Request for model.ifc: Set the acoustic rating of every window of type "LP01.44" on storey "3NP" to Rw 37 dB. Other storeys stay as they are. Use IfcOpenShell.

First a look at what the model holds.

```python
import ifcopenshell
import ifcopenshell.util.element

model = ifcopenshell.open("model.ifc")
print(model.schema)
storey = next(s for s in model.by_type("IfcBuildingStorey") if s.Name == "3NP")
windows = [e for e in ifcopenshell.util.element.get_decomposition(storey) if e.is_a("IfcWindow")]
seen = {}
for e in windows:
    element_type = ifcopenshell.util.element.get_type(e)
    key = (element_type.Name if element_type != e and element_type else None, ifcopenshell.util.element.get_pset(e, "Pset_WindowCommon", "AcousticRating"))
    seen[key] = seen.get(key, 0) + 1
for (name, value), count in sorted(seen.items(), key=str):
    print(count, "x", name, "|", value)
```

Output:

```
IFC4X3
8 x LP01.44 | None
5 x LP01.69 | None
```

```python
import ifcopenshell
import ifcopenshell.api.pset
import ifcopenshell.util.element

model = ifcopenshell.open("model.ifc")

storey = next(s for s in model.by_type("IfcBuildingStorey") if s.Name == "3NP")
windows = [e for e in ifcopenshell.util.element.get_decomposition(storey) if e.is_a("IfcWindow")]

count = 0
for e in windows:
    element_type = ifcopenshell.util.element.get_type(e)
    if element_type in (None, e) or element_type.Name != "LP01.44":
        continue
    # add_pset returns the element's existing set when there is one.
    pset = ifcopenshell.api.pset.add_pset(model, product=e, name="Pset_WindowCommon")
    ifcopenshell.api.pset.edit_pset(model, pset=pset, properties={"AcousticRating": "Rw 37 dB"})
    count += 1

print(count, "windows updated")

model.write("model_rev.ifc")
```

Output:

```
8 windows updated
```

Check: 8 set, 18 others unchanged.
